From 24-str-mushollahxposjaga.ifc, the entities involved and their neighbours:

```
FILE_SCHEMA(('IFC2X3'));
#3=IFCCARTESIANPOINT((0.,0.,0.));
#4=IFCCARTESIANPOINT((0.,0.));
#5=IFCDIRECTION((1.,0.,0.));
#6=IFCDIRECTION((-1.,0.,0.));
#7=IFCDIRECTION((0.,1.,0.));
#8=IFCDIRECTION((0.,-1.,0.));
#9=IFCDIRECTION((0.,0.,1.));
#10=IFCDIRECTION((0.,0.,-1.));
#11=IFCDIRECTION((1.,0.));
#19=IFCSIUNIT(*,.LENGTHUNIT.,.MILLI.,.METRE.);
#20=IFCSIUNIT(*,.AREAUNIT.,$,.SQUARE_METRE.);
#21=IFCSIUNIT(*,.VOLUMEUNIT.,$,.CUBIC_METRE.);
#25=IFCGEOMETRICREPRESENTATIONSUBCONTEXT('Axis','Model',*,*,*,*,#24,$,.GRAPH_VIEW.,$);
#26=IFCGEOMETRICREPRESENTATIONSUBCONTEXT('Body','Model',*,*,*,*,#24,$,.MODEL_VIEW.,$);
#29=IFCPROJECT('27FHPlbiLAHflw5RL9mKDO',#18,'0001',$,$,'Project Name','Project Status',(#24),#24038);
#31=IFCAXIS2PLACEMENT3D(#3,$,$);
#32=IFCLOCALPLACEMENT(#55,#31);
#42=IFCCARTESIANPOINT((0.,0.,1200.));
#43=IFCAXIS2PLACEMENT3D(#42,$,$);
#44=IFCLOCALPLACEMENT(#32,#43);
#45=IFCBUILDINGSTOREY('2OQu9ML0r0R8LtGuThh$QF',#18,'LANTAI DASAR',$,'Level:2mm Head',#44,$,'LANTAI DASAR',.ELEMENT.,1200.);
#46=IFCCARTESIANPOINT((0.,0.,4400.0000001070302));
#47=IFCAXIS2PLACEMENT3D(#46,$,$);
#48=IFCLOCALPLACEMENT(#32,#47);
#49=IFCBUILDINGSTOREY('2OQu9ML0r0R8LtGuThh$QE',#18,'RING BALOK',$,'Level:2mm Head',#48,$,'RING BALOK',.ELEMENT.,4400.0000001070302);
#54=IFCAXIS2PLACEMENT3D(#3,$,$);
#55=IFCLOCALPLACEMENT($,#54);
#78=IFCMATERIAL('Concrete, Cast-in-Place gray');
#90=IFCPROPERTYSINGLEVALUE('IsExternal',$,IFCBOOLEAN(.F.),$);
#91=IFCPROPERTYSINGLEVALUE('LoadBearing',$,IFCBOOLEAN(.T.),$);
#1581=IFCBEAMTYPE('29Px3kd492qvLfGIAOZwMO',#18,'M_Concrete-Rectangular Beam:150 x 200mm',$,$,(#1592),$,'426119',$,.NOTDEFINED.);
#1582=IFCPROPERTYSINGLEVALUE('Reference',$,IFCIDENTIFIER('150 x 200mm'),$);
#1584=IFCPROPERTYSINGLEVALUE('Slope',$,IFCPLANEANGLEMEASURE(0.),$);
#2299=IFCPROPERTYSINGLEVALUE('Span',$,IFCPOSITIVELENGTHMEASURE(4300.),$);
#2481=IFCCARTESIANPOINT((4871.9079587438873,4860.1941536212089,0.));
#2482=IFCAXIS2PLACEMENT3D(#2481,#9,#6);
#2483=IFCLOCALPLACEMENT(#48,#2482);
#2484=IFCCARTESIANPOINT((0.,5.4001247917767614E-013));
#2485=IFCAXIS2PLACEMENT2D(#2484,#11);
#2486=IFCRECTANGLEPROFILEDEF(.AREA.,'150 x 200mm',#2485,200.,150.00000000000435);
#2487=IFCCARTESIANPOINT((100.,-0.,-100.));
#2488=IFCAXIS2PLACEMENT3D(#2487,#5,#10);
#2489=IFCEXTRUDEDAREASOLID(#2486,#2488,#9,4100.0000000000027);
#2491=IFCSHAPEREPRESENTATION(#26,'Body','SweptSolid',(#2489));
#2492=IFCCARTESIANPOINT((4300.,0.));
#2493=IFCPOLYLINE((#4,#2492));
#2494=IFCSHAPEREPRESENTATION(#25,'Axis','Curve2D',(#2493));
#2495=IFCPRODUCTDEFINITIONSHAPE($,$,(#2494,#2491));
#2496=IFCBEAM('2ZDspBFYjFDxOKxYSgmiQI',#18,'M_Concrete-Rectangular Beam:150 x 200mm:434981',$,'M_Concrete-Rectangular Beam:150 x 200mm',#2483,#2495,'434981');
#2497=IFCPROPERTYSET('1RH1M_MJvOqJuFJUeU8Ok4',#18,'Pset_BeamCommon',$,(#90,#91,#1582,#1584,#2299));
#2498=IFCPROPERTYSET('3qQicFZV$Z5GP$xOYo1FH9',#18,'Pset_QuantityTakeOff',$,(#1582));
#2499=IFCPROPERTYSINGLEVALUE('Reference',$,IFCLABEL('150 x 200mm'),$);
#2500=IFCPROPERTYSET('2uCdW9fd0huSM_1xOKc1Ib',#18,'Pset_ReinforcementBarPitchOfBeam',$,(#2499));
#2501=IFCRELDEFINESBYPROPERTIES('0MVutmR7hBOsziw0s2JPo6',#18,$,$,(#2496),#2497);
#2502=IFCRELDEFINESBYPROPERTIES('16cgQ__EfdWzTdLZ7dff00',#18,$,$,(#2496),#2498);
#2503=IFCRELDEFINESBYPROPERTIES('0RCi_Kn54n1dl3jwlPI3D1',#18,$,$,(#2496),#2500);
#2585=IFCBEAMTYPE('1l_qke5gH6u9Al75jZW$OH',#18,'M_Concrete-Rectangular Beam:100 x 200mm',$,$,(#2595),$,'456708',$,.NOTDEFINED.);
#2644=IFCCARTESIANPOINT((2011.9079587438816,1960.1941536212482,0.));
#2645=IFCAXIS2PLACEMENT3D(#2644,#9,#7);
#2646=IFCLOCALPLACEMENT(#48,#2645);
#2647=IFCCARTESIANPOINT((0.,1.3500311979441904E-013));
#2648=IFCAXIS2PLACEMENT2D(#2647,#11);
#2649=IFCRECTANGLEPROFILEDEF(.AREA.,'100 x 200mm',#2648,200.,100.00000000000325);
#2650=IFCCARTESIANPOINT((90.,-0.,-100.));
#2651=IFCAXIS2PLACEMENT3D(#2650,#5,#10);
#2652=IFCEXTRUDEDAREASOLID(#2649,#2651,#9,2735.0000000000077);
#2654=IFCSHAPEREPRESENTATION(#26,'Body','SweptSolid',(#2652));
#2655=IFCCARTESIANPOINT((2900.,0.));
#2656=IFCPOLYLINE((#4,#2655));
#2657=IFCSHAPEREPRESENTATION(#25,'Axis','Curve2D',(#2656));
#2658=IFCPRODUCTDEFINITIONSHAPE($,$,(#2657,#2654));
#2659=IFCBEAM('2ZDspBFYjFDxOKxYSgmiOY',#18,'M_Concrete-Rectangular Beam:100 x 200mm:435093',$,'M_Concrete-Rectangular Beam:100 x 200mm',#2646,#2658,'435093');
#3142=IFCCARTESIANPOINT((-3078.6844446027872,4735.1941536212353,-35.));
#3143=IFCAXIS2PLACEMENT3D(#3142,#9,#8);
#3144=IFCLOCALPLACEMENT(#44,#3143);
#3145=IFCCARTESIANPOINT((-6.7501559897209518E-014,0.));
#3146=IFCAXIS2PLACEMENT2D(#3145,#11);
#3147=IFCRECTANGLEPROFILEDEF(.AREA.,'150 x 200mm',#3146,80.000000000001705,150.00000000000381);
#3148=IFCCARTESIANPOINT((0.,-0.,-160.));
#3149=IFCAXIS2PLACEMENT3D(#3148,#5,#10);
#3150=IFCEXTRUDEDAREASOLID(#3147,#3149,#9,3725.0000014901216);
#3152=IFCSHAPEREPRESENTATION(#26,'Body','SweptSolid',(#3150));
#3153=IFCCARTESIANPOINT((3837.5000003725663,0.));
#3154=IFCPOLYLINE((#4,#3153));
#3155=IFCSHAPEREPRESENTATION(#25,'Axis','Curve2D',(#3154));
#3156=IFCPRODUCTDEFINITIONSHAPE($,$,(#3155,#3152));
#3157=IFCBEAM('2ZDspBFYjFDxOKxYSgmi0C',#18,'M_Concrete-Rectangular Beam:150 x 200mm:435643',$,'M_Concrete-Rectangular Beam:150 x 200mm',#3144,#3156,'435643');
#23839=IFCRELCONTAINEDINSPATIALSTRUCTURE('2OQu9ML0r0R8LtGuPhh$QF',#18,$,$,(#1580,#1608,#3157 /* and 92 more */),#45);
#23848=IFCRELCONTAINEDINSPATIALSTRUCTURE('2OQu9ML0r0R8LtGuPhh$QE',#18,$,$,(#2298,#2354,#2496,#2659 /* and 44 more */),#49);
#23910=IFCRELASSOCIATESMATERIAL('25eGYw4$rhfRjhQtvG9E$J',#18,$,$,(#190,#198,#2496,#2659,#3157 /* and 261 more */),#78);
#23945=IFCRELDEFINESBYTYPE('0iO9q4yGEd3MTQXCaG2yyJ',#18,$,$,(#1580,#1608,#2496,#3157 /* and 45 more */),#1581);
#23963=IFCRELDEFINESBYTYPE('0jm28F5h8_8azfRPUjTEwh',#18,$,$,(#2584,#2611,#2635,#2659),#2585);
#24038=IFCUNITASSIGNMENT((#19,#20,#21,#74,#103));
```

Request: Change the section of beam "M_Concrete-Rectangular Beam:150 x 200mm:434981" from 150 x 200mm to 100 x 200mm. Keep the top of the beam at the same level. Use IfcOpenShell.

```python
import ifcopenshell
import ifcopenshell.api.pset
import ifcopenshell.api.type
import ifcopenshell.util.element
import ifcopenshell.util.representation

model = ifcopenshell.open("24-str-mushollahxposjaga.ifc")

member = model.by_guid("2ZDspBFYjFDxOKxYSgmiQI")
source = next(p for p in model.by_type("IfcRectangleProfileDef") if p.ProfileName == "100 x 200mm")

body = ifcopenshell.util.representation.get_representation(member, "Model", "Body")
solid = body.Items[0]
old_profile = solid.SweptArea

# Copy the section's sizes but keep this member's own profile position.
profile = ifcopenshell.util.element.copy(model, source)
# Profiles are centred, so shift by half the change in depth to hold the top.
shift = (old_profile.XDim - profile.XDim) / 2
x, y = old_profile.Position.Location.Coordinates
up = (-1.0, 0.0)  # upwards, in the solid's own plane
location = model.createIfcCartesianPoint((x + up[0] * shift, y + up[1] * shift))
profile.Position = model.createIfcAxis2Placement2D(location, old_profile.Position.RefDirection)
solid.SweptArea = profile
if not model.get_total_inverses(old_profile):
    ifcopenshell.util.element.remove_deep2(model, old_profile)

new_type = model.by_guid("1l_qke5gH6u9Al75jZW$OH")
ifcopenshell.api.type.assign_type(
    model, related_objects=[member], relating_type=new_type, should_map_representations=False
)
member.Name = member.Name.replace("150 x 200mm", "100 x 200mm")
member.ObjectType = "M_Concrete-Rectangular Beam:100 x 200mm"
pset = model.by_id(ifcopenshell.util.element.get_pset(member, "Pset_BeamCommon", should_inherit=False)["id"])
ifcopenshell.api.pset.edit_pset(model, pset=pset, properties={"Reference": "100 x 200mm"})
pset = model.by_id(ifcopenshell.util.element.get_pset(member, "Pset_QuantityTakeOff", should_inherit=False)["id"])
ifcopenshell.api.pset.edit_pset(model, pset=pset, properties={"Reference": "100 x 200mm"})
pset = model.by_id(ifcopenshell.util.element.get_pset(member, "Pset_ReinforcementBarPitchOfBeam", should_inherit=False)["id"])
ifcopenshell.api.pset.edit_pset(model, pset=pset, properties={"Reference": "100 x 200mm"})

print(solid.SweptArea)

model.write("24-str-mushollahxposjaga_edited.ifc")
```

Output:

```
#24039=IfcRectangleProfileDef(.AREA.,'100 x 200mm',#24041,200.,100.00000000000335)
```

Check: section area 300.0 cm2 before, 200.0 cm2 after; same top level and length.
